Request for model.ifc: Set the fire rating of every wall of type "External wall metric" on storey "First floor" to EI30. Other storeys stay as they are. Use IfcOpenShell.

First a look at what the model holds.

```python
import ifcopenshell
import ifcopenshell.util.element

model = ifcopenshell.open("model.ifc")
print(model.schema)
storey = next(s for s in model.by_type("IfcBuildingStorey") if s.Name == "First floor")
walls = [e for e in ifcopenshell.util.element.get_decomposition(storey) if e.is_a("IfcWall")]
seen = {}
for e in walls:
    element_type = ifcopenshell.util.element.get_type(e)
    key = (element_type.Name if element_type != e and element_type else None, ifcopenshell.util.element.get_pset(e, "Pset_WallCommon", "FireRating"))
    seen[key] = seen.get(key, 0) + 1
for (name, value), count in sorted(seen.items(), key=str):
    print(count, "x", name, "|", value)
```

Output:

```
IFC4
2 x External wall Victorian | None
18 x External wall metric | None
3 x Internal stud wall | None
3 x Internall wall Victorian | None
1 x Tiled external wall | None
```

```python
import ifcopenshell
import ifcopenshell.api.pset
import ifcopenshell.util.element

model = ifcopenshell.open("model.ifc")

storey = next(s for s in model.by_type("IfcBuildingStorey") if s.Name == "First floor")
walls = [e for e in ifcopenshell.util.element.get_decomposition(storey) if e.is_a("IfcWall")]

count = 0
for e in walls:
    element_type = ifcopenshell.util.element.get_type(e)
    if element_type in (None, e) or element_type.Name != "External wall metric":
        continue
    # add_pset returns the element's existing set when there is one.
    pset = ifcopenshell.api.pset.add_pset(model, product=e, name="Pset_WallCommon")
    ifcopenshell.api.pset.edit_pset(model, pset=pset, properties={"FireRating": "EI30"})
    count += 1

print(count, "walls updated")

model.write("model-out.ifc")
```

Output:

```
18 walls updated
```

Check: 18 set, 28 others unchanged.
